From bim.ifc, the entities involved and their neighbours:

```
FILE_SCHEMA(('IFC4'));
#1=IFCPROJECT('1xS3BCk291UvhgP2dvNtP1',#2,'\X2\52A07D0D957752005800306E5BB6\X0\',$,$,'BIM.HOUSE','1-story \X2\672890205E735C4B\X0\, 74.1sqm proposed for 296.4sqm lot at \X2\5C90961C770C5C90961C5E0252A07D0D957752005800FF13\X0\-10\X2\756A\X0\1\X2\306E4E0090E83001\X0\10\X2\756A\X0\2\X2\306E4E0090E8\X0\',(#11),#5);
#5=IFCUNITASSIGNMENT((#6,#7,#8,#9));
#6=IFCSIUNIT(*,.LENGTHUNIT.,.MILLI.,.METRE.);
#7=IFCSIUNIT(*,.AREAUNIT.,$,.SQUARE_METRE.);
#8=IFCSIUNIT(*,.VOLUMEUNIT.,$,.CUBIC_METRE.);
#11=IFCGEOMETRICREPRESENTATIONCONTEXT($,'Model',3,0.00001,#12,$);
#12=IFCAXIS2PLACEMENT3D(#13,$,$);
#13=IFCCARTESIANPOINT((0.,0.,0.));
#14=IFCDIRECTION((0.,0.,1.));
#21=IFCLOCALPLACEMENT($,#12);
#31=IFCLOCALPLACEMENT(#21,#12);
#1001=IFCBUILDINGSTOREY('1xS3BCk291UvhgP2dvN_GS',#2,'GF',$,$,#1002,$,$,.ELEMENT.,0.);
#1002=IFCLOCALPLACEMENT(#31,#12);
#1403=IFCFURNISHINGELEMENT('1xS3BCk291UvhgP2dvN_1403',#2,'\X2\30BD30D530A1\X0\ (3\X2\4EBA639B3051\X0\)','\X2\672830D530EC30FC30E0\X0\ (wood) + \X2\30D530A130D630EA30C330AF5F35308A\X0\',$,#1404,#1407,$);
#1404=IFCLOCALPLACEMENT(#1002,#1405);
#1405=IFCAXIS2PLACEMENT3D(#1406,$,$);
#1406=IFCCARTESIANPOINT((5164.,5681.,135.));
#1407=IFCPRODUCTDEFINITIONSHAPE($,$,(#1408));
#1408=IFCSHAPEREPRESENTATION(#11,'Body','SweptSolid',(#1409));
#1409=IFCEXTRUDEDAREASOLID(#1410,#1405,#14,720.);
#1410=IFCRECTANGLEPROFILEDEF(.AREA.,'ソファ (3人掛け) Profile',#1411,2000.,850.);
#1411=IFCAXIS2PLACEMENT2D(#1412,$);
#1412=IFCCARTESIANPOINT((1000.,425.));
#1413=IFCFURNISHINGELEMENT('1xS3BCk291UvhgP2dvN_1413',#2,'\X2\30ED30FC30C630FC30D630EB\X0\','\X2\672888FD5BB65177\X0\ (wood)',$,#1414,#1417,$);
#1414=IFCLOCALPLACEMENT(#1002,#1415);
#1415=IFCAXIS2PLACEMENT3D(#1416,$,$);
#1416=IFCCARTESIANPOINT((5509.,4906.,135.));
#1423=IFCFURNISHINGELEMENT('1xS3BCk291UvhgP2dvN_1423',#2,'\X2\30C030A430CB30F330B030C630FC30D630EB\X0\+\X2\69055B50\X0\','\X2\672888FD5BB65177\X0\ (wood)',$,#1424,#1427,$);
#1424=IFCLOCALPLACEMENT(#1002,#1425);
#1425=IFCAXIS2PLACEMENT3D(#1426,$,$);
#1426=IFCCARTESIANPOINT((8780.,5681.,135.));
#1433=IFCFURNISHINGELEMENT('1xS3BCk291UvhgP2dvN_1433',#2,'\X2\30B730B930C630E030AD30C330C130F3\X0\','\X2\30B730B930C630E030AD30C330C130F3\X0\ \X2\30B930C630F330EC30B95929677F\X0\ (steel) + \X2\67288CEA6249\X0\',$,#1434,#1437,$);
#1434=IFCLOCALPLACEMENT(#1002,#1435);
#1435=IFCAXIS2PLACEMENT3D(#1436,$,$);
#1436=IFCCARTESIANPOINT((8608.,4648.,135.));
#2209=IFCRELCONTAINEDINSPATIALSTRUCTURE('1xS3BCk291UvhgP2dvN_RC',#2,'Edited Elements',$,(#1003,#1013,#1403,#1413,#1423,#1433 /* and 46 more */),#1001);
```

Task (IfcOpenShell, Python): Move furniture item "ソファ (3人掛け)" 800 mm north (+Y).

```python
import ifcopenshell
import ifcopenshell.api.geometry
import ifcopenshell.util.placement
import ifcopenshell.util.unit

model = ifcopenshell.open("bim.ifc")
unit_scale = ifcopenshell.util.unit.calculate_unit_scale(model)

item = model.by_guid("1xS3BCk291UvhgP2dvN_1403")
matrix = ifcopenshell.util.placement.get_local_placement(item.ObjectPlacement)
matrix[1, 3] += 0.8 / unit_scale
ifcopenshell.api.geometry.edit_object_placement(model, product=item, matrix=matrix, is_si=False)

print(ifcopenshell.util.placement.get_local_placement(item.ObjectPlacement).round(3) + 0.0)

model.write("bim_rev.ifc")
```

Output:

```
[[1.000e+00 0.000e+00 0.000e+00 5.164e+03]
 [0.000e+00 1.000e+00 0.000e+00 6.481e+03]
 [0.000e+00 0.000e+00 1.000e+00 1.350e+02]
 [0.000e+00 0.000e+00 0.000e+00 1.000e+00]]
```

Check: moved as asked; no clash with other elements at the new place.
